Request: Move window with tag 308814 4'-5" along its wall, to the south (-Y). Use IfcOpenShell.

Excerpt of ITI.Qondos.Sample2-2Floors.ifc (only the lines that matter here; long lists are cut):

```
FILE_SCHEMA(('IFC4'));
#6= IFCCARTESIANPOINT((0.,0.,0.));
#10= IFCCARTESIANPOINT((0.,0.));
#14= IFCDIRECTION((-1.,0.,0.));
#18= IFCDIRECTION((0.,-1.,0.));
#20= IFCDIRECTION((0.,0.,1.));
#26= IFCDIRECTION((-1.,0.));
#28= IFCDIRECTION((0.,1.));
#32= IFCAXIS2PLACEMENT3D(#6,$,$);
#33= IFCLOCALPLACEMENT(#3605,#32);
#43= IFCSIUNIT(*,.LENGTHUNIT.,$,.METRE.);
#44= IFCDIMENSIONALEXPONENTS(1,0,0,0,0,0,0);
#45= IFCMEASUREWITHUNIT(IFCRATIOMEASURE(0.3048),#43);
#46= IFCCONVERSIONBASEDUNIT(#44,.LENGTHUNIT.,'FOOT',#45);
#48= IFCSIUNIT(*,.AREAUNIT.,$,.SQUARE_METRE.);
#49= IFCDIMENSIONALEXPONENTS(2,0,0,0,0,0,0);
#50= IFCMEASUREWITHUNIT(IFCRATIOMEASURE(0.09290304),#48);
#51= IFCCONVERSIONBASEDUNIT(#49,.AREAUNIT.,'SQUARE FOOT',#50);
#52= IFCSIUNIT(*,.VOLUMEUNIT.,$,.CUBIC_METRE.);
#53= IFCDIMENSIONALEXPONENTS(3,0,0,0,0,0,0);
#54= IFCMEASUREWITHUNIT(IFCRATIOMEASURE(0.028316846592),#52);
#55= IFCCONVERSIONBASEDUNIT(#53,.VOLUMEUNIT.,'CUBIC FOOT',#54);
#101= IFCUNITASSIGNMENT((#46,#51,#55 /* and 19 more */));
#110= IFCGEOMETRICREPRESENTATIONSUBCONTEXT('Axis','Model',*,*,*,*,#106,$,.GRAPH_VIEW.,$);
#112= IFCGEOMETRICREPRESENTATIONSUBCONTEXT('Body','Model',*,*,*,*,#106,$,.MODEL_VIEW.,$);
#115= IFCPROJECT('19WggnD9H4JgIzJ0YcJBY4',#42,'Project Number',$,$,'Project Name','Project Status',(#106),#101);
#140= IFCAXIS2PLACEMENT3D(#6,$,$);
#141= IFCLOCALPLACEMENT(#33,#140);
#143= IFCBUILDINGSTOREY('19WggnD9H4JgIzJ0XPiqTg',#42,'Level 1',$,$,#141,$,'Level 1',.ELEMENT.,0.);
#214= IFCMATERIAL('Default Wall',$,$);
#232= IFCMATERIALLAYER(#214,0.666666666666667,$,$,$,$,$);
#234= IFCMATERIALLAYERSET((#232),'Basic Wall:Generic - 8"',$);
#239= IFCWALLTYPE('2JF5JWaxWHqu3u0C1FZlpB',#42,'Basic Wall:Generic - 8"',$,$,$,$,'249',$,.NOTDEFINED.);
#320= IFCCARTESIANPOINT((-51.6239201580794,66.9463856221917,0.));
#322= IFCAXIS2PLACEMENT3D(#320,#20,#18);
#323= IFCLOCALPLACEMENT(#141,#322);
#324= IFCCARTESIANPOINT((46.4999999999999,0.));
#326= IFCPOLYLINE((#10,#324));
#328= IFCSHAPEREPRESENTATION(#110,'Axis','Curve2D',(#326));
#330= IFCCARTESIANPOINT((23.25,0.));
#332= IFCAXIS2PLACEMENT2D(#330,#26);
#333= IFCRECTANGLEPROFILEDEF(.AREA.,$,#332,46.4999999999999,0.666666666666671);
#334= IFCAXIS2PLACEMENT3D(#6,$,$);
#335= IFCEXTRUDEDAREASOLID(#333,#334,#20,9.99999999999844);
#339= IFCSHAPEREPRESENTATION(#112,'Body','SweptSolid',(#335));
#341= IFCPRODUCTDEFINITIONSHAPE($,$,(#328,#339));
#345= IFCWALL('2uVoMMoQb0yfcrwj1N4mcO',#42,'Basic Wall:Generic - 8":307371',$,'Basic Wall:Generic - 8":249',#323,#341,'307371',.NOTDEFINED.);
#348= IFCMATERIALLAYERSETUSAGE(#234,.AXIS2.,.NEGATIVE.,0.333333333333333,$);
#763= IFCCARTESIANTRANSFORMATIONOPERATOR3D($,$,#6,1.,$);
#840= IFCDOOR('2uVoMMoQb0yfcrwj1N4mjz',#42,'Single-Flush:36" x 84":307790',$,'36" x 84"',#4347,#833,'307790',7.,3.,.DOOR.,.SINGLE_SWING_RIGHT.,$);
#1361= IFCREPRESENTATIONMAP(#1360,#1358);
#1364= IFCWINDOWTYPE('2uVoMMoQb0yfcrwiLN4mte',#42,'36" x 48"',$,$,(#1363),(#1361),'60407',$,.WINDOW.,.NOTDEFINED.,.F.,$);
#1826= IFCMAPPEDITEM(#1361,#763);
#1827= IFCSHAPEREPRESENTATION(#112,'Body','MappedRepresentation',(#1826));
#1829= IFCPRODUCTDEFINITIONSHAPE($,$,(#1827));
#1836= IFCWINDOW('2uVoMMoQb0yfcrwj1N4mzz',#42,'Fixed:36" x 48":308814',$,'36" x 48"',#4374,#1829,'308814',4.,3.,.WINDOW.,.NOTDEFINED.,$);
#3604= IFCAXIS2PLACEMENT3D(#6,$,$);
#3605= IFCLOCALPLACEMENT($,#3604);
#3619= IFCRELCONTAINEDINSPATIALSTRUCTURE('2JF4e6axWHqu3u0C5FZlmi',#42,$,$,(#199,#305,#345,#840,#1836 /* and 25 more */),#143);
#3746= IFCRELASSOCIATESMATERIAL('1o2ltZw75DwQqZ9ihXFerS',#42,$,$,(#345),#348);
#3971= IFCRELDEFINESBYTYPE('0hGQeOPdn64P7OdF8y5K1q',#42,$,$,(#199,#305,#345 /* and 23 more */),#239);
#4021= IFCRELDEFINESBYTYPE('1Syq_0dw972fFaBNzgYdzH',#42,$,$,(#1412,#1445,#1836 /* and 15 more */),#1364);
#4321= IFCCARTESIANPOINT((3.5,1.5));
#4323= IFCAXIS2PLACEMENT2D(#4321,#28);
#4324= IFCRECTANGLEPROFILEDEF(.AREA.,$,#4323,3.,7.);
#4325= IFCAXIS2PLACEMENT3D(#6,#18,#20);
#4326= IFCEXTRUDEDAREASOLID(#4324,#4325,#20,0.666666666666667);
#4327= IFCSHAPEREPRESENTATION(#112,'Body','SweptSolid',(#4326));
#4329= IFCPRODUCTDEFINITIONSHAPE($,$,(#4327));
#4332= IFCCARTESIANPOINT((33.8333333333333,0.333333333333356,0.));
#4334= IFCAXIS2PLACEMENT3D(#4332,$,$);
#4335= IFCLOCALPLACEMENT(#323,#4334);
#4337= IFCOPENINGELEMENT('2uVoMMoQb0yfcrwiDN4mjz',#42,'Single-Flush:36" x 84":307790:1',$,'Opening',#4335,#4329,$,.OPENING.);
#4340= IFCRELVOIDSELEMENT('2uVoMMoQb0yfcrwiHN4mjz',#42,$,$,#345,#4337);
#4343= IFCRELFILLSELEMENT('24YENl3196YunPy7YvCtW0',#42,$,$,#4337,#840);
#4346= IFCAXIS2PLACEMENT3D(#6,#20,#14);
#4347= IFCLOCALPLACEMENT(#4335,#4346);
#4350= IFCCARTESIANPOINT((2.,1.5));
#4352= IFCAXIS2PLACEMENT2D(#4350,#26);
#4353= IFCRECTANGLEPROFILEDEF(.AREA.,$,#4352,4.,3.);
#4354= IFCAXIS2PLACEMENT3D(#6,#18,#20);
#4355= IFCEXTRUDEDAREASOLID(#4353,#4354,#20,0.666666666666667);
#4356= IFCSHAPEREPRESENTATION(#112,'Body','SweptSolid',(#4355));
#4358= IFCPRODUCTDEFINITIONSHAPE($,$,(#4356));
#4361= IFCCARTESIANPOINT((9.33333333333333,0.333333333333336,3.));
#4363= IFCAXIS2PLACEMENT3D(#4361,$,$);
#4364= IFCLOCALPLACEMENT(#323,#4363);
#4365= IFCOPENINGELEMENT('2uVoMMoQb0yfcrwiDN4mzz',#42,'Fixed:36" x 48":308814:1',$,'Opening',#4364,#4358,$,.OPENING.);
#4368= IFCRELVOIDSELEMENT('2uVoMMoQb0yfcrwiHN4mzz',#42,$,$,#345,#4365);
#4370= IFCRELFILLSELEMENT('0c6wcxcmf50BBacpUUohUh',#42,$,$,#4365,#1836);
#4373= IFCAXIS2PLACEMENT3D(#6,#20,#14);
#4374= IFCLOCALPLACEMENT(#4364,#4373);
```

```python
import ifcopenshell
import ifcopenshell.api.geometry
import ifcopenshell.util.placement
import ifcopenshell.util.unit

model = ifcopenshell.open("ITI.Qondos.Sample2-2Floors.ifc")
unit_scale = ifcopenshell.util.unit.calculate_unit_scale(model)

window = model.by_guid("2uVoMMoQb0yfcrwj1N4mzz")
opening = window.FillsVoids[0].RelatingOpeningElement
wall = opening.VoidsElements[0].RelatingBuildingElement

wall_matrix = ifcopenshell.util.placement.get_local_placement(wall.ObjectPlacement)
shift = wall_matrix[:3, 0] * 53 * 0.0254 / unit_scale
before = ifcopenshell.util.placement.get_local_placement(window.ObjectPlacement)[:3, 3].copy()

# The window is placed relative to its opening, so it follows when the opening moves.
matrix = ifcopenshell.util.placement.get_local_placement(opening.ObjectPlacement)
matrix[:3, 3] += shift
ifcopenshell.api.geometry.edit_object_placement(
    model, product=opening, matrix=matrix, is_si=False, should_transform_children=True
)

after = ifcopenshell.util.placement.get_local_placement(window.ObjectPlacement)[:3, 3]
print("window moved by", (after - before).round(3) + 0.0)

model.write("ITI.Qondos.Sample2-2Floors_updated.ifc")
```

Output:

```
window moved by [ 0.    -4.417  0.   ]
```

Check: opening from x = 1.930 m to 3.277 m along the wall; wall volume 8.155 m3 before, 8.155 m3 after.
